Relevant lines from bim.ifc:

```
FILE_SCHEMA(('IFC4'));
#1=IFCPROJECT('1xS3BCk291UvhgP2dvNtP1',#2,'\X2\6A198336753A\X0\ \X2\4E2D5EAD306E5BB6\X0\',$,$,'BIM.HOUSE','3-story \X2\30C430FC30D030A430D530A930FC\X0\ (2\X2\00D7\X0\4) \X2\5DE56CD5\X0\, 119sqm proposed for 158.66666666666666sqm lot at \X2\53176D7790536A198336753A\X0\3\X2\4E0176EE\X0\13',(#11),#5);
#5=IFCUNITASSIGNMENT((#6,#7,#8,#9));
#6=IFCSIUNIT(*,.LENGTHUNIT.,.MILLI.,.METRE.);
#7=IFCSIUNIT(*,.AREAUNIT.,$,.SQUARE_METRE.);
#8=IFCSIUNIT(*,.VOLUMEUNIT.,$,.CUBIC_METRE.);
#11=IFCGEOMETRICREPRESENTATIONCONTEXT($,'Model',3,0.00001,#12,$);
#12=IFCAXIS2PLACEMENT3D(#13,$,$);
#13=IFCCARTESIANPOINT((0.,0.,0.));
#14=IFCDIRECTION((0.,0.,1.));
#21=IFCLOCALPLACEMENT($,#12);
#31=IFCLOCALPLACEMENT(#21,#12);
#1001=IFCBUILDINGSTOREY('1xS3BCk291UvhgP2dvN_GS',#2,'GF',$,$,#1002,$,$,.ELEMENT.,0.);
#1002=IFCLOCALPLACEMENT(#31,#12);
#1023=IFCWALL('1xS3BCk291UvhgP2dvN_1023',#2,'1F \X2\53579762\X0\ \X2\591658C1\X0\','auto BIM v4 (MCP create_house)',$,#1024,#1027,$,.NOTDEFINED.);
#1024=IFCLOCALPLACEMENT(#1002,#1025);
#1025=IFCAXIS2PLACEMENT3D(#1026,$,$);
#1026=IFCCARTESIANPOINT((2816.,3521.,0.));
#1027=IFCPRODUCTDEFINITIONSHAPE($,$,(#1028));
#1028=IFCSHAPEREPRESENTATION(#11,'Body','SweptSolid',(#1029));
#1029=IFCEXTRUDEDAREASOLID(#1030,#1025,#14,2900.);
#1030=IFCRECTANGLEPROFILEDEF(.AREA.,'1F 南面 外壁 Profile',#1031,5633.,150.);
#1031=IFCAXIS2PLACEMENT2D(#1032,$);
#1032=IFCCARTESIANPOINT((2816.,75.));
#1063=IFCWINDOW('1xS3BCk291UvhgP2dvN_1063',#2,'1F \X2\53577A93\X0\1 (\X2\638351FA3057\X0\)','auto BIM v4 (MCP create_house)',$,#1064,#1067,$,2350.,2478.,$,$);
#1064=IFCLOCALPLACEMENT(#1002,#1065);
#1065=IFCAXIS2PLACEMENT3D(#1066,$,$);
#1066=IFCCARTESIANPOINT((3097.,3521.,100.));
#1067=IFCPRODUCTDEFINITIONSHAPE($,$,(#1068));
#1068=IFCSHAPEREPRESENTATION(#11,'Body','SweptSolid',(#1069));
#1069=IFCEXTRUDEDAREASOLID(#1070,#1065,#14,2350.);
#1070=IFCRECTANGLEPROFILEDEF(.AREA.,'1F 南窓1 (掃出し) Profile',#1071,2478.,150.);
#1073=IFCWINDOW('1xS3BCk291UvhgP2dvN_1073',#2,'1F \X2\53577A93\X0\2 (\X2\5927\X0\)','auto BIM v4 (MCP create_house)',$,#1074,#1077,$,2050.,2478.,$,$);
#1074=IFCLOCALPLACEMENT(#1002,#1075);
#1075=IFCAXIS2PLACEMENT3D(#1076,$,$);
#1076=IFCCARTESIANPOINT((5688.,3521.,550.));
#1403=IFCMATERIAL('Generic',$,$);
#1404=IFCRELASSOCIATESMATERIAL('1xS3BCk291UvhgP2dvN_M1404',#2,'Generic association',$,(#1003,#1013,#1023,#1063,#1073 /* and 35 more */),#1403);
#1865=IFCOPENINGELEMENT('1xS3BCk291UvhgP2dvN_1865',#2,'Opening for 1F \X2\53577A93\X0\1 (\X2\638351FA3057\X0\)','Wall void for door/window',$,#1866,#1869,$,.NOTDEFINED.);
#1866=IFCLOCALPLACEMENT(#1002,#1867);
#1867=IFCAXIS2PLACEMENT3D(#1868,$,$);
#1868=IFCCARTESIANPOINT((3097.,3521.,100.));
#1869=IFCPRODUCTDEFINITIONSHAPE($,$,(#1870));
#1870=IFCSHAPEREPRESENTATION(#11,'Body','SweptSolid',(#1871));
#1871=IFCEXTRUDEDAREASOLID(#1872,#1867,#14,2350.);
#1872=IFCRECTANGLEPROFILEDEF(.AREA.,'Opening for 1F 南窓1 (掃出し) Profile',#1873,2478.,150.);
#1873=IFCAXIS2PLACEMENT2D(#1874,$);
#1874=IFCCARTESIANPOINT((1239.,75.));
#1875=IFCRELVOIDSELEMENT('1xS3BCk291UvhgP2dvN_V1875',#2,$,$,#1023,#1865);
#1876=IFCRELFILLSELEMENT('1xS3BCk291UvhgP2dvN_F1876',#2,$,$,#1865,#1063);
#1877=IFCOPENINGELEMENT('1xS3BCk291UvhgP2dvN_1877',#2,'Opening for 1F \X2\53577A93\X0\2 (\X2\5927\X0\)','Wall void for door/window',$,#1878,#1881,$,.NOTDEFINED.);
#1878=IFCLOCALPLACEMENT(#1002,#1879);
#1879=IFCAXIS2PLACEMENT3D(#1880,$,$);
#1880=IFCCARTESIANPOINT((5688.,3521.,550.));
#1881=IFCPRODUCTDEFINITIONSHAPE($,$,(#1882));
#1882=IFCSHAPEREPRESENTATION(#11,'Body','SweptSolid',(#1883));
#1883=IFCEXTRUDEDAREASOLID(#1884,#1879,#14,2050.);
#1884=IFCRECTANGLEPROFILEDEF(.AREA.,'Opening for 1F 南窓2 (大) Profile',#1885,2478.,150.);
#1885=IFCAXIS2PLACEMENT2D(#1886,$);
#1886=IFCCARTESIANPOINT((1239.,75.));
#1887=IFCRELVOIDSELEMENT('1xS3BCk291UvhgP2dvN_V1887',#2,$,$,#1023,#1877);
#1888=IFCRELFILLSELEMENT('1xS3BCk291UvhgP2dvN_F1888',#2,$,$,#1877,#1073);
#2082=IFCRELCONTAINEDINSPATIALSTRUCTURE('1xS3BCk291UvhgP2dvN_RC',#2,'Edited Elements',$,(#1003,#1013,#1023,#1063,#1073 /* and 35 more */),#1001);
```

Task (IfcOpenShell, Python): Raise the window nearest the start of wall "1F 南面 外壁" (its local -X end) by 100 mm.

```python
import numpy as np
import ifcopenshell
import ifcopenshell.api.geometry
import ifcopenshell.util.placement
import ifcopenshell.util.unit

model = ifcopenshell.open("bim.ifc")
unit_scale = ifcopenshell.util.unit.calculate_unit_scale(model)

window = model.by_guid("1xS3BCk291UvhgP2dvN_1063")
opening = window.FillsVoids[0].RelatingOpeningElement
dz = 100.0

shift = np.array([0.0, 0.0, dz])
# The window is not placed relative to its opening, so move both.
for product in (opening, window):
    matrix = ifcopenshell.util.placement.get_local_placement(product.ObjectPlacement)
    matrix[:3, 3] += shift
    ifcopenshell.api.geometry.edit_object_placement(model, product=product, matrix=matrix, is_si=False)

print(f"moved by {dz * unit_scale:+.3f} m")

model.write("bim_rev.ifc")
```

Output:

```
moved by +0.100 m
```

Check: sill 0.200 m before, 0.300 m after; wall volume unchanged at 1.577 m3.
